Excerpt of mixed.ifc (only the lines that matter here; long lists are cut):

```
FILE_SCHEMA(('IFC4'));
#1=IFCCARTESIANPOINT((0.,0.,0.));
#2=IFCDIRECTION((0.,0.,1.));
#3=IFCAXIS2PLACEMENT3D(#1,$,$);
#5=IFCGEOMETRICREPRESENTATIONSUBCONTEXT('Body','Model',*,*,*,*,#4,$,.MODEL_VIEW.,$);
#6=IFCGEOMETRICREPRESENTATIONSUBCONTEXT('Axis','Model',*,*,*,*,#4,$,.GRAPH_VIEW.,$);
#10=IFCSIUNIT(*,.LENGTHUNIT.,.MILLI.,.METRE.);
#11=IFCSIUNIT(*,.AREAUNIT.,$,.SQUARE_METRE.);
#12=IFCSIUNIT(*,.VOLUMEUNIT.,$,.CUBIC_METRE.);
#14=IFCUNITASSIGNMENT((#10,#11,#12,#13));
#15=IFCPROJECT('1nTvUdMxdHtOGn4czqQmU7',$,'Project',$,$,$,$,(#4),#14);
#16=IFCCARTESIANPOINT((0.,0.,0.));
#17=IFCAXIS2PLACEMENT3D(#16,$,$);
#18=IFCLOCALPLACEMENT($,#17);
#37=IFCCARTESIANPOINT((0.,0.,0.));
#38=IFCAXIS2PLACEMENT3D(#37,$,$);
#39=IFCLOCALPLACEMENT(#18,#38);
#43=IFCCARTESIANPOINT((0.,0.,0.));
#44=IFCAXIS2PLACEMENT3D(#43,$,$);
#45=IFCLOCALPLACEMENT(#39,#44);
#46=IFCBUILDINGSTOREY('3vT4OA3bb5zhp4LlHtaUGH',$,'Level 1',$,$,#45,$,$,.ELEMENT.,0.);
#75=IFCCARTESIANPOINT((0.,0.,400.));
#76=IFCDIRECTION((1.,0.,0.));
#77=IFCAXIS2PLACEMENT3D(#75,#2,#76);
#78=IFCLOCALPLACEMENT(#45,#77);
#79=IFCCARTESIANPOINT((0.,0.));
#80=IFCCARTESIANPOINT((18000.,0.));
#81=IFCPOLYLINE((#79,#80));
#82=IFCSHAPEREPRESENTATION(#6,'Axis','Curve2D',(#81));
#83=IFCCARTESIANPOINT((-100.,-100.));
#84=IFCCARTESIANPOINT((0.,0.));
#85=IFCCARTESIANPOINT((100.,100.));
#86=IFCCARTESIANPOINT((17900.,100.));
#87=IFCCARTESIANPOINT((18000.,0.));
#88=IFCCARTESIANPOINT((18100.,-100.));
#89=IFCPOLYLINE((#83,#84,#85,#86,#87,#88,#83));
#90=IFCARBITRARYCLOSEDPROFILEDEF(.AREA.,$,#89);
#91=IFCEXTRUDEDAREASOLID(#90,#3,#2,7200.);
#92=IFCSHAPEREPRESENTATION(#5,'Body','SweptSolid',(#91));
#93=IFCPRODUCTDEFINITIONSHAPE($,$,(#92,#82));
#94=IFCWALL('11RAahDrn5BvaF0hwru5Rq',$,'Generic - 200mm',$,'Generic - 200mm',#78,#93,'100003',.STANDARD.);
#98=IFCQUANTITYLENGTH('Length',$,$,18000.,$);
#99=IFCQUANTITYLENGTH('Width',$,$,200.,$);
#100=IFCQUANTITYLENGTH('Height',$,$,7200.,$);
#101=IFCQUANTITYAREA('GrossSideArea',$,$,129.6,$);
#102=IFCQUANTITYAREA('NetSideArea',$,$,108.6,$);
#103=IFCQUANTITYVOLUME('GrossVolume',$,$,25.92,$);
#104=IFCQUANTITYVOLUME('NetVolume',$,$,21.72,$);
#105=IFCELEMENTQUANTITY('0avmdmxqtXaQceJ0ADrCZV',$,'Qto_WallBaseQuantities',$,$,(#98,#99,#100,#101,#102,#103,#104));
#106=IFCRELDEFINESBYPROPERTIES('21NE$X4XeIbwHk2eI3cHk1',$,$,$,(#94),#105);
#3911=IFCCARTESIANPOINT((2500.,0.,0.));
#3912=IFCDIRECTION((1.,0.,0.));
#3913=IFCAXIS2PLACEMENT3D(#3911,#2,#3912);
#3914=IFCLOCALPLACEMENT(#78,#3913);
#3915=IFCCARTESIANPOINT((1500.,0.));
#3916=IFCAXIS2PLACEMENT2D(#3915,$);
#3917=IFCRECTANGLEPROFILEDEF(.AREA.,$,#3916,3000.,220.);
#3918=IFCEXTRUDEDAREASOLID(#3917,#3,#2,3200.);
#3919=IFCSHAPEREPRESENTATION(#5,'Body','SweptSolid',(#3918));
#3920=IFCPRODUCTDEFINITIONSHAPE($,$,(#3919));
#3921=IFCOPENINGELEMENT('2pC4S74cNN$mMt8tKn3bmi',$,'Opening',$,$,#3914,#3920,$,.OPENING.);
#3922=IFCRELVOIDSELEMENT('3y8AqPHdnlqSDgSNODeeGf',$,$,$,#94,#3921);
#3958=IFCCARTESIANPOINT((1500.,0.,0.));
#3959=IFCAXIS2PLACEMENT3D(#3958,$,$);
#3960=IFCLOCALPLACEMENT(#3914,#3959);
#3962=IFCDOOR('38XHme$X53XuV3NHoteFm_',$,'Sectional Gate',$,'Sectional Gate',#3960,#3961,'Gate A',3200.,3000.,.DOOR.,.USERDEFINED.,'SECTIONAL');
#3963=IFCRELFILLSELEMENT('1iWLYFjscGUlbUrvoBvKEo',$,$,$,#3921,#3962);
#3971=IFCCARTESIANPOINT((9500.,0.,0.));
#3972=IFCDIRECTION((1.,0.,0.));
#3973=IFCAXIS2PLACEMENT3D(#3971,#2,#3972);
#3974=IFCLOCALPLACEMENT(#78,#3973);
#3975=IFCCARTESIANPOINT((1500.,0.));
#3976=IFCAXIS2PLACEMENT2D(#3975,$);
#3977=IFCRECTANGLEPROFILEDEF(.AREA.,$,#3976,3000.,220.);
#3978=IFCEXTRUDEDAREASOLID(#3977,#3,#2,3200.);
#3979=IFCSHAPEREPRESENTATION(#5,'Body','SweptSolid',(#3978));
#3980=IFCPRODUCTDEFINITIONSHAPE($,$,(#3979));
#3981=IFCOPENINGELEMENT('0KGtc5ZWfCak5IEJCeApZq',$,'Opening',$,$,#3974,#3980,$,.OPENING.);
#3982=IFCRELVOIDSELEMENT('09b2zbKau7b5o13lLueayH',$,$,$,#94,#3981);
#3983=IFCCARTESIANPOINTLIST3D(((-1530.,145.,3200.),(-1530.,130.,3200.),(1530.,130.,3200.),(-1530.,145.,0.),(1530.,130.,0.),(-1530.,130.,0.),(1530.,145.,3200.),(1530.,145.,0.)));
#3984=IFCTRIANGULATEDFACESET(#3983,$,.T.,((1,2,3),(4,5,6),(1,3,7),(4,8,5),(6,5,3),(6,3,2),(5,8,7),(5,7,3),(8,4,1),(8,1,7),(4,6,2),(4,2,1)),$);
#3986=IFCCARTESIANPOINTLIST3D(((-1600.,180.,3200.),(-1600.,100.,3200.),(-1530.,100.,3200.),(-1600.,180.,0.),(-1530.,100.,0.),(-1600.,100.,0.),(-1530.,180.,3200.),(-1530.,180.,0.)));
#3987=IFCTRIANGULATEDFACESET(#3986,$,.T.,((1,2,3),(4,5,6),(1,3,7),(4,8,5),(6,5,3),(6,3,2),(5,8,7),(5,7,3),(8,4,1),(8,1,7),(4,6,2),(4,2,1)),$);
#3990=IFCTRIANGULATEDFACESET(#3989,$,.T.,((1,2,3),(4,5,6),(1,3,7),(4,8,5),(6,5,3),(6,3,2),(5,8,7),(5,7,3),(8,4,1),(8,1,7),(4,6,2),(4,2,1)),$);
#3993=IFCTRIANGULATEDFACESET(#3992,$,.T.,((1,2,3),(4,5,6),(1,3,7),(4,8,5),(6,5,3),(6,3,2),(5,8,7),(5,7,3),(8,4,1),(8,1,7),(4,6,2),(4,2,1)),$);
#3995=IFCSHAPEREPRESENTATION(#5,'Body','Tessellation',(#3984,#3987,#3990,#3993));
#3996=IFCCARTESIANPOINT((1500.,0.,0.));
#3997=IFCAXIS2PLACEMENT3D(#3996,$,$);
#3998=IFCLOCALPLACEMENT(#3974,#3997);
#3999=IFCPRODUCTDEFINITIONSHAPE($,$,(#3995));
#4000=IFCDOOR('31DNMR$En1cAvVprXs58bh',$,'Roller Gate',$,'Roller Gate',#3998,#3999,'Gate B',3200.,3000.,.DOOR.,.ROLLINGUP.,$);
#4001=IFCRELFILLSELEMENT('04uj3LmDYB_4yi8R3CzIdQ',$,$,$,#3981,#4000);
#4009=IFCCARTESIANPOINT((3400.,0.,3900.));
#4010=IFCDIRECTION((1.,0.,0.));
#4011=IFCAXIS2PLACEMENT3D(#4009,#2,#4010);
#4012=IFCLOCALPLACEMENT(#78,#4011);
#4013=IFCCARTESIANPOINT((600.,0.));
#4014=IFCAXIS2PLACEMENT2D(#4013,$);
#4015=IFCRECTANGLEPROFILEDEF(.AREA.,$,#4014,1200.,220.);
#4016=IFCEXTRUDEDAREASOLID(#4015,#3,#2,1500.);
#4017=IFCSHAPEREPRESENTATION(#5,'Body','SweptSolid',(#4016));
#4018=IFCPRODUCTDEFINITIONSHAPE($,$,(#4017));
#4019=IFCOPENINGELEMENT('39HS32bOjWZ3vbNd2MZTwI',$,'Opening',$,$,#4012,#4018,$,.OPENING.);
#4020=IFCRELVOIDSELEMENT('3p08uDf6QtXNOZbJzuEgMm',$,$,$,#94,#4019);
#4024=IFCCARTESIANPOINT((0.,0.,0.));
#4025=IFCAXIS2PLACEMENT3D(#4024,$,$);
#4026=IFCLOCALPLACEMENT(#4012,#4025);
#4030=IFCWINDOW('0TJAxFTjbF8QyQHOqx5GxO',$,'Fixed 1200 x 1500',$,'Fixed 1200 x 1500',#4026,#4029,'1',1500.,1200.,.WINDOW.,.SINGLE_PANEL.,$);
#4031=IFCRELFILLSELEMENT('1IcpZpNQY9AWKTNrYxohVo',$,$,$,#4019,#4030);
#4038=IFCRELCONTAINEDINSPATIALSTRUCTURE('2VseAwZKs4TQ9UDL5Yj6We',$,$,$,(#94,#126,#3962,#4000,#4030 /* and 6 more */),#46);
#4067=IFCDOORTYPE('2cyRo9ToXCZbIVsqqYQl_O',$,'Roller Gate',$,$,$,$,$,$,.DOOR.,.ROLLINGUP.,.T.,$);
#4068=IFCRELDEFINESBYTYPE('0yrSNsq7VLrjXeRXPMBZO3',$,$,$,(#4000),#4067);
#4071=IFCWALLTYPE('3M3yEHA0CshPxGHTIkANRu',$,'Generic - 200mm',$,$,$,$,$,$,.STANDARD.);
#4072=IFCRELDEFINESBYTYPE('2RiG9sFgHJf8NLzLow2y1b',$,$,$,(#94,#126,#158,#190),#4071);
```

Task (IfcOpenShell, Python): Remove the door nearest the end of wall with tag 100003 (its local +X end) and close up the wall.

```python
import ifcopenshell
import ifcopenshell.api.feature
import ifcopenshell.api.pset
import ifcopenshell.api.root
import ifcopenshell.geom
import ifcopenshell.util.element
import ifcopenshell.util.shape
import ifcopenshell.util.unit

model = ifcopenshell.open("mixed.ifc")
area_scale = ifcopenshell.util.unit.calculate_unit_scale(model, "AREAUNIT")
volume_scale = ifcopenshell.util.unit.calculate_unit_scale(model, "VOLUMEUNIT")
settings = ifcopenshell.geom.settings()


def volume(element):
    """Net volume in cubic metres, openings subtracted."""
    shape = ifcopenshell.geom.create_shape(settings, element)
    return ifcopenshell.util.shape.get_volume(shape.geometry)


door = model.by_guid("31DNMR$En1cAvVprXs58bh")
opening = door.FillsVoids[0].RelatingOpeningElement
wall = opening.VoidsElements[0].RelatingBuildingElement
before = volume(wall)

ifcopenshell.api.root.remove_product(model, product=door)
ifcopenshell.api.feature.remove_feature(model, feature=opening)

after = volume(wall)
thickness = 0.2  # wall thickness in metres

# Update the wall's stored quantities.
qto = model.by_id(ifcopenshell.util.element.get_pset(wall, "Qto_WallBaseQuantities", should_inherit=False)["id"])
ifcopenshell.api.pset.edit_qto(model, qto=qto, properties={
    "NetSideArea": after / thickness / area_scale,
    "NetVolume": after / volume_scale,
})

print(f"wall volume {before:.3f} -> {after:.3f} m3")

model.write("mixed-out.ifc")
```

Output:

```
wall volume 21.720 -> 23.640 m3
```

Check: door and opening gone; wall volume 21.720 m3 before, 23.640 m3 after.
